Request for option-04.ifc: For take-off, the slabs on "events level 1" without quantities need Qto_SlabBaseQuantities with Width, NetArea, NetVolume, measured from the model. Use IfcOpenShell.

First a look at what the model holds.

```python
import ifcopenshell
import ifcopenshell.util.element
import ifcopenshell.util.unit

model = ifcopenshell.open("option-04.ifc")
print(model.schema)
for unit_type in ("LENGTHUNIT", "AREAUNIT", "VOLUMEUNIT"):
    print(unit_type, ifcopenshell.util.unit.calculate_unit_scale(model, unit_type))
storey = next(s for s in model.by_type("IfcBuildingStorey") if s.Name == "events level 1")
slabs = [e for e in ifcopenshell.util.element.get_decomposition(storey) if e.is_a("IfcSlab")]
for e in sorted(slabs, key=lambda e: e.id()):
    print(e.id(), e.is_a(), e.Name, list(ifcopenshell.util.element.get_psets(e, qtos_only=True)), sep=" | ")
```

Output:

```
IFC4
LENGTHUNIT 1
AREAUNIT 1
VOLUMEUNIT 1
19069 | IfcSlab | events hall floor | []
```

```python
import ifcopenshell
import ifcopenshell.api.pset
import ifcopenshell.geom
import ifcopenshell.util.element
import ifcopenshell.util.shape
import ifcopenshell.util.unit

model = ifcopenshell.open("option-04.ifc")
unit_scale = ifcopenshell.util.unit.calculate_unit_scale(model)
area_scale = ifcopenshell.util.unit.calculate_unit_scale(model, "AREAUNIT")
volume_scale = ifcopenshell.util.unit.calculate_unit_scale(model, "VOLUMEUNIT")
settings = ifcopenshell.geom.settings()

storey = next(s for s in model.by_type("IfcBuildingStorey") if s.Name == "events level 1")
slabs = [e for e in ifcopenshell.util.element.get_decomposition(storey) if e.is_a("IfcSlab")]

for e in sorted(slabs, key=lambda e: e.id()):
    if ifcopenshell.util.element.get_psets(e, qtos_only=True, should_inherit=False):
        continue
    # Geometry comes back in metres, in the element's own axes.
    shape = ifcopenshell.geom.create_shape(settings, e)
    values = {
        "Width": ifcopenshell.util.shape.get_z(shape.geometry) / unit_scale,
        "NetArea": ifcopenshell.util.shape.get_footprint_area(shape.geometry) / area_scale,
        "NetVolume": ifcopenshell.util.shape.get_volume(shape.geometry) / volume_scale,
    }
    qto = ifcopenshell.api.pset.add_qto(model, product=e, name="Qto_SlabBaseQuantities")
    ifcopenshell.api.pset.edit_qto(model, qto=qto, properties=values)
    print(e.id(), {k: round(v, 3) for k, v in values.items()})

model.write("option-04_v2.ifc")
```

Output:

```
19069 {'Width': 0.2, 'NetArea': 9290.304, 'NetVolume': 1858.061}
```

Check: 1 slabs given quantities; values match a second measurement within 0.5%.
